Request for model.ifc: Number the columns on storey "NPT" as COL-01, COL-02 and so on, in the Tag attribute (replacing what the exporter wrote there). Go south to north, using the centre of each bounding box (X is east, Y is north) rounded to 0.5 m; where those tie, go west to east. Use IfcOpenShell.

First a look at what the model holds.

```python
import ifcopenshell
import ifcopenshell.util.element
import ifcopenshell.util.placement

model = ifcopenshell.open("model.ifc")
print(model.schema)
storey = next(s for s in model.by_type("IfcBuildingStorey") if s.Name == "NPT")
columns = [e for e in ifcopenshell.util.element.get_decomposition(storey) if e.is_a("IfcColumn")]
for e in sorted(columns, key=lambda e: e.id()):
    origin = ifcopenshell.util.placement.get_local_placement(e.ObjectPlacement)[:3, 3]
    print(e.id(), e.Tag, e.Name, origin.round(2) + 0.0, sep=" | ")
```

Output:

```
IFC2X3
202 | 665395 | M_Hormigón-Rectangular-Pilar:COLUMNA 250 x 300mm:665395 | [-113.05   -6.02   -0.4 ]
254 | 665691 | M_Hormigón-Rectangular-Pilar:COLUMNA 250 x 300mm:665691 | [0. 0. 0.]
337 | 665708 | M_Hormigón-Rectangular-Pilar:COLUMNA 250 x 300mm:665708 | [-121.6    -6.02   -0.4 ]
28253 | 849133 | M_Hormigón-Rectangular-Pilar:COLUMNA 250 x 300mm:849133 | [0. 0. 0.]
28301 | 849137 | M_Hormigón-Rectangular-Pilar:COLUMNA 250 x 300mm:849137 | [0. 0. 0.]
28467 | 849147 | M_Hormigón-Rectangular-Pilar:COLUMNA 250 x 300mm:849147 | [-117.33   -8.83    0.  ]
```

```python
import ifcopenshell
import ifcopenshell.geom
import ifcopenshell.util.element
import ifcopenshell.util.shape

model = ifcopenshell.open("model.ifc")
settings = ifcopenshell.geom.settings()
settings.set("use-world-coords", True)


def centre(element):
    shape = ifcopenshell.geom.create_shape(settings, element)
    return ifcopenshell.util.shape.get_bbox_centroid(shape.geometry)


storey = next(s for s in model.by_type("IfcBuildingStorey") if s.Name == "NPT")
columns = [e for e in ifcopenshell.util.element.get_decomposition(storey) if e.is_a("IfcColumn")]

# Insertion points can sit at a corner or the storey origin, so sort by the geometry (in metres).
centres = {e: centre(e) for e in columns}
columns.sort(key=lambda e: (round(centres[e][1] / 0.5), centres[e][0]))

for i, e in enumerate(columns, start=1):
    number = f"COL-{i:02d}"
    e.Tag = number
    print(e.id(), number)

model.write("model_updated.ifc")
```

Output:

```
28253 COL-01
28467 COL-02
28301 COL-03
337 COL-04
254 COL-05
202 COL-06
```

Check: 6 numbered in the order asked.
